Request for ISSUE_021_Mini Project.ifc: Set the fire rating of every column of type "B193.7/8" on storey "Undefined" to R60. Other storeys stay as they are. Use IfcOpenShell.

First a look at what the model holds.

```python
import ifcopenshell
import ifcopenshell.util.element

model = ifcopenshell.open("ISSUE_021_Mini Project.ifc")
print(model.schema)
storey = next(s for s in model.by_type("IfcBuildingStorey") if s.Name == "Undefined")
columns = [e for e in ifcopenshell.util.element.get_decomposition(storey) if e.is_a("IfcColumn")]
seen = {}
for e in columns:
    element_type = ifcopenshell.util.element.get_type(e)
    key = (element_type.Name if element_type != e and element_type else None, ifcopenshell.util.element.get_pset(e, "Pset_ColumnCommon", "FireRating"))
    seen[key] = seen.get(key, 0) + 1
for (name, value), count in sorted(seen.items(), key=str):
    print(count, "x", name, "|", value)
```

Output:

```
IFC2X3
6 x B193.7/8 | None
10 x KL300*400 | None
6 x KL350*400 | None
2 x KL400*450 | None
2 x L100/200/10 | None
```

```python
import ifcopenshell
import ifcopenshell.api.pset
import ifcopenshell.util.element

model = ifcopenshell.open("ISSUE_021_Mini Project.ifc")

storey = next(s for s in model.by_type("IfcBuildingStorey") if s.Name == "Undefined")
columns = [e for e in ifcopenshell.util.element.get_decomposition(storey) if e.is_a("IfcColumn")]

count = 0
for e in columns:
    element_type = ifcopenshell.util.element.get_type(e)
    if element_type in (None, e) or element_type.Name != "B193.7/8":
        continue
    found = ifcopenshell.util.element.get_pset(e, "Pset_ColumnCommon", should_inherit=False)
    if found:
        pset = model.by_id(found["id"])
        if len(ifcopenshell.util.element.get_elements_by_pset(pset)) > 1:
            pset = ifcopenshell.api.pset.unshare_pset(model, products=[e], pset=pset)[0]
    else:
        pset = ifcopenshell.api.pset.add_pset(model, product=e, name="Pset_ColumnCommon")
    ifcopenshell.api.pset.edit_pset(model, pset=pset, properties={"FireRating": "R60"})
    count += 1

print(count, "columns updated")

model.write("ISSUE_021_Mini Project_updated.ifc")
```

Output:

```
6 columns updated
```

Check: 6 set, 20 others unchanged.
